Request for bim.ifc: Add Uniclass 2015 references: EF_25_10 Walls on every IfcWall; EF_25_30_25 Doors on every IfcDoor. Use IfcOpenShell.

First a look at what the model holds.

```python
import ifcopenshell

model = ifcopenshell.open("bim.ifc")
print(model.schema)
print("classifications:", [c.Name for c in model.by_type("IfcClassification")])
for ifc_class in ("IfcDoor", "IfcRoof", "IfcStair", "IfcWall", "IfcWindow"):
    print(ifc_class, len(model.by_type(ifc_class)))
```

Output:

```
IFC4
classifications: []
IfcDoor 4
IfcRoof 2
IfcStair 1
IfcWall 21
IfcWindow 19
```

```python
import ifcopenshell
import ifcopenshell.api.classification

model = ifcopenshell.open("bim.ifc")

system = ifcopenshell.api.classification.add_classification(model, classification="Uniclass 2015")

codes = {
    "IfcWall": ("EF_25_10", "Walls"),
    "IfcDoor": ("EF_25_30_25", "Doors"),
}
for ifc_class, (code, name) in codes.items():
    products = model.by_type(ifc_class)
    ifcopenshell.api.classification.add_reference(
        model, products=products, classification=system, identification=code, name=name
    )
    print(code, len(products))

model.write("bim_updated.ifc")
```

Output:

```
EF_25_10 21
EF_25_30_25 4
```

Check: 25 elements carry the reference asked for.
